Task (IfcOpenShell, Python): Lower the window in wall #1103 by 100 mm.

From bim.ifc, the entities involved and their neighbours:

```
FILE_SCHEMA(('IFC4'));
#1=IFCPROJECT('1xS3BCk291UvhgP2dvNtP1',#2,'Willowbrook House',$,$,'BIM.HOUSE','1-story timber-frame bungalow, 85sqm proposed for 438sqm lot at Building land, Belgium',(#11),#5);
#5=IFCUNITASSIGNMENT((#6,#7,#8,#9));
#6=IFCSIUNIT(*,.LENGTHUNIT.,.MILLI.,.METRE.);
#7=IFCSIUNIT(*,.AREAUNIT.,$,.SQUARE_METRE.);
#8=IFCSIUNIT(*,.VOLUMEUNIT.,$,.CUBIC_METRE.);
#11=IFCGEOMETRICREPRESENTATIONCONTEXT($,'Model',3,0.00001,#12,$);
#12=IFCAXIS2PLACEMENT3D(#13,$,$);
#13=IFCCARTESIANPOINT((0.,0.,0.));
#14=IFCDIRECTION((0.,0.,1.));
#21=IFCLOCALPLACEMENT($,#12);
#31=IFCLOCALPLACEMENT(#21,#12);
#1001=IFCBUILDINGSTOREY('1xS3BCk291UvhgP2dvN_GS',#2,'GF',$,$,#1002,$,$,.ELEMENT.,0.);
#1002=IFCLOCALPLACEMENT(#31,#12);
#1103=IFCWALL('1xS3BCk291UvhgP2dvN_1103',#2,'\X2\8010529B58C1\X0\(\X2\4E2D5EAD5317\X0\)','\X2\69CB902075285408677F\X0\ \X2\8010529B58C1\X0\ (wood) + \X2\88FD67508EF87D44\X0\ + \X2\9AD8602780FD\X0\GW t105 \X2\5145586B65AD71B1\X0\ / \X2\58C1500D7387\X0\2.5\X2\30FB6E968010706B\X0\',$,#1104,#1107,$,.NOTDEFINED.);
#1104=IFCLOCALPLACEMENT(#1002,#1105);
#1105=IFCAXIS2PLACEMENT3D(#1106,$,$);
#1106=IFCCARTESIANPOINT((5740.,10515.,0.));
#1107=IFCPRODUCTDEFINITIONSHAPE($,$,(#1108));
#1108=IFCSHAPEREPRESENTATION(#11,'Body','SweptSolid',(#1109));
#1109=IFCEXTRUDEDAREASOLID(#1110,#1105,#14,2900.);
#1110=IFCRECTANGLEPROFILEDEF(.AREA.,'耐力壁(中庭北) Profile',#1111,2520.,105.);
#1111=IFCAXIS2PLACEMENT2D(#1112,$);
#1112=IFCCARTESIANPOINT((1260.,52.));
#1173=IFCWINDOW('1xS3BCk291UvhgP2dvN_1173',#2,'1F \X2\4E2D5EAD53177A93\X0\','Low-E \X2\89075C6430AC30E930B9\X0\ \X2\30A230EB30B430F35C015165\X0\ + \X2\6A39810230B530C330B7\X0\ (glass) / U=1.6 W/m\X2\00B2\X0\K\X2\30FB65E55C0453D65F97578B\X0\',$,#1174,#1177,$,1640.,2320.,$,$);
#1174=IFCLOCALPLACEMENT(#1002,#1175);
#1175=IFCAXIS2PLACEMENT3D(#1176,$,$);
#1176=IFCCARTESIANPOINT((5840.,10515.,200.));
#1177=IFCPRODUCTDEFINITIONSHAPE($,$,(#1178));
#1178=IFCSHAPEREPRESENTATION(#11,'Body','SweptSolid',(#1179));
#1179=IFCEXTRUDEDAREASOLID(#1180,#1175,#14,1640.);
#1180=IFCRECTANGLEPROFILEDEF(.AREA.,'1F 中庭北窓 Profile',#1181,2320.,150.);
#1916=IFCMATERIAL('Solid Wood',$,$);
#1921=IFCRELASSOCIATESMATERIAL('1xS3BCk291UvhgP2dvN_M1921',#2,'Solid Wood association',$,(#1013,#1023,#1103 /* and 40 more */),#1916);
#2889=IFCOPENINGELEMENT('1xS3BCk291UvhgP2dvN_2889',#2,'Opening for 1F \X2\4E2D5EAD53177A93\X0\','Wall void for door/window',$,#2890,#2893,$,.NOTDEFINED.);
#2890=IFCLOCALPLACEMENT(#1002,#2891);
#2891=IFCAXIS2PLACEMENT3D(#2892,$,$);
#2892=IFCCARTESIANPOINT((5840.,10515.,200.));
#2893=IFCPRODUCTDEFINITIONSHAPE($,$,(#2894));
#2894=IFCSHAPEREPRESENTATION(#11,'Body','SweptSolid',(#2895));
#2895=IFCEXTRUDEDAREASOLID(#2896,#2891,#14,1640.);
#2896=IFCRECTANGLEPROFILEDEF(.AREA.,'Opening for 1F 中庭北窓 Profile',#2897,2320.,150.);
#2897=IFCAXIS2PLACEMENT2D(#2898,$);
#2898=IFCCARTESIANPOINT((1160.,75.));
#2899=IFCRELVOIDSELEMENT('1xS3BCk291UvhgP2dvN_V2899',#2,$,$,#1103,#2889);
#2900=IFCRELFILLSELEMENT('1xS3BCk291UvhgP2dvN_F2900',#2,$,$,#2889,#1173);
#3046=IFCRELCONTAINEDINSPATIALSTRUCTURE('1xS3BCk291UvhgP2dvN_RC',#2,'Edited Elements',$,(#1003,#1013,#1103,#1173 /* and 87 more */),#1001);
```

```python
import numpy as np
import ifcopenshell
import ifcopenshell.api.geometry
import ifcopenshell.util.placement
import ifcopenshell.util.unit

model = ifcopenshell.open("bim.ifc")
unit_scale = ifcopenshell.util.unit.calculate_unit_scale(model)

window = model.by_guid("1xS3BCk291UvhgP2dvN_1173")
opening = window.FillsVoids[0].RelatingOpeningElement
dz = -0.1 / unit_scale

shift = np.array([0.0, 0.0, dz])
# The window is not placed relative to its opening, so move both.
for product in (opening, window):
    matrix = ifcopenshell.util.placement.get_local_placement(product.ObjectPlacement)
    matrix[:3, 3] += shift
    ifcopenshell.api.geometry.edit_object_placement(model, product=product, matrix=matrix, is_si=False)

print(f"moved by {dz * unit_scale:+.3f} m")

model.write("bim-out.ifc")
```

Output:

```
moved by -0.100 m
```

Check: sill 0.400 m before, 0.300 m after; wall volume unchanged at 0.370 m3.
